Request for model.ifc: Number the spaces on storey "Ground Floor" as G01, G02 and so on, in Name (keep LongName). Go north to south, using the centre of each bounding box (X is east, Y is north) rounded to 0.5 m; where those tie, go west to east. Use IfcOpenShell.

First a look at what the model holds.

```python
import ifcopenshell
import ifcopenshell.util.element
import ifcopenshell.util.placement

model = ifcopenshell.open("model.ifc")
print(model.schema)
storey = next(s for s in model.by_type("IfcBuildingStorey") if s.Name == "Ground Floor")
spaces = [e for e in ifcopenshell.util.element.get_decomposition(storey) if e.is_a("IfcSpace")]
for e in sorted(spaces, key=lambda e: e.id()):
    origin = ifcopenshell.util.placement.get_local_placement(e.ObjectPlacement)[:3, 3]
    print(e.id(), e.Name, e.LongName, origin.round(2) + 0.0, sep=" | ")
```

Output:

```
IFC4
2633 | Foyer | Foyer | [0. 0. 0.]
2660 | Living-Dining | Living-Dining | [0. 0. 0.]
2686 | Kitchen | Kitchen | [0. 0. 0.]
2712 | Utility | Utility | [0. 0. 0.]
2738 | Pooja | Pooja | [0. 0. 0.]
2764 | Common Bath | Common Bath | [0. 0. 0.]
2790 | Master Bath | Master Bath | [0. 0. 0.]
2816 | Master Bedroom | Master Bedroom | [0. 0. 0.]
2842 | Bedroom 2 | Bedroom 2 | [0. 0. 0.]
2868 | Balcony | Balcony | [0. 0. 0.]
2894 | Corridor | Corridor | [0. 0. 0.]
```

```python
import ifcopenshell
import ifcopenshell.geom
import ifcopenshell.util.element
import ifcopenshell.util.shape

model = ifcopenshell.open("model.ifc")
settings = ifcopenshell.geom.settings()
settings.set("use-world-coords", True)


def centre(element):
    shape = ifcopenshell.geom.create_shape(settings, element)
    return ifcopenshell.util.shape.get_bbox_centroid(shape.geometry)


storey = next(s for s in model.by_type("IfcBuildingStorey") if s.Name == "Ground Floor")
spaces = [e for e in ifcopenshell.util.element.get_decomposition(storey) if e.is_a("IfcSpace")]

# Insertion points can sit at a corner or the storey origin, so sort by the geometry (in metres).
centres = {e: centre(e) for e in spaces}
spaces.sort(key=lambda e: (-round(centres[e][1] / 0.5), centres[e][0]))

for i, e in enumerate(spaces, start=1):
    number = f"G{i:02d}"
    e.Name = number
    print(e.id(), number)

model.write("model_v2.ifc")
```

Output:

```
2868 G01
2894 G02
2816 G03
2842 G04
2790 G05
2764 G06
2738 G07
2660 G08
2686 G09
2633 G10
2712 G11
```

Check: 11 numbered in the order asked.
